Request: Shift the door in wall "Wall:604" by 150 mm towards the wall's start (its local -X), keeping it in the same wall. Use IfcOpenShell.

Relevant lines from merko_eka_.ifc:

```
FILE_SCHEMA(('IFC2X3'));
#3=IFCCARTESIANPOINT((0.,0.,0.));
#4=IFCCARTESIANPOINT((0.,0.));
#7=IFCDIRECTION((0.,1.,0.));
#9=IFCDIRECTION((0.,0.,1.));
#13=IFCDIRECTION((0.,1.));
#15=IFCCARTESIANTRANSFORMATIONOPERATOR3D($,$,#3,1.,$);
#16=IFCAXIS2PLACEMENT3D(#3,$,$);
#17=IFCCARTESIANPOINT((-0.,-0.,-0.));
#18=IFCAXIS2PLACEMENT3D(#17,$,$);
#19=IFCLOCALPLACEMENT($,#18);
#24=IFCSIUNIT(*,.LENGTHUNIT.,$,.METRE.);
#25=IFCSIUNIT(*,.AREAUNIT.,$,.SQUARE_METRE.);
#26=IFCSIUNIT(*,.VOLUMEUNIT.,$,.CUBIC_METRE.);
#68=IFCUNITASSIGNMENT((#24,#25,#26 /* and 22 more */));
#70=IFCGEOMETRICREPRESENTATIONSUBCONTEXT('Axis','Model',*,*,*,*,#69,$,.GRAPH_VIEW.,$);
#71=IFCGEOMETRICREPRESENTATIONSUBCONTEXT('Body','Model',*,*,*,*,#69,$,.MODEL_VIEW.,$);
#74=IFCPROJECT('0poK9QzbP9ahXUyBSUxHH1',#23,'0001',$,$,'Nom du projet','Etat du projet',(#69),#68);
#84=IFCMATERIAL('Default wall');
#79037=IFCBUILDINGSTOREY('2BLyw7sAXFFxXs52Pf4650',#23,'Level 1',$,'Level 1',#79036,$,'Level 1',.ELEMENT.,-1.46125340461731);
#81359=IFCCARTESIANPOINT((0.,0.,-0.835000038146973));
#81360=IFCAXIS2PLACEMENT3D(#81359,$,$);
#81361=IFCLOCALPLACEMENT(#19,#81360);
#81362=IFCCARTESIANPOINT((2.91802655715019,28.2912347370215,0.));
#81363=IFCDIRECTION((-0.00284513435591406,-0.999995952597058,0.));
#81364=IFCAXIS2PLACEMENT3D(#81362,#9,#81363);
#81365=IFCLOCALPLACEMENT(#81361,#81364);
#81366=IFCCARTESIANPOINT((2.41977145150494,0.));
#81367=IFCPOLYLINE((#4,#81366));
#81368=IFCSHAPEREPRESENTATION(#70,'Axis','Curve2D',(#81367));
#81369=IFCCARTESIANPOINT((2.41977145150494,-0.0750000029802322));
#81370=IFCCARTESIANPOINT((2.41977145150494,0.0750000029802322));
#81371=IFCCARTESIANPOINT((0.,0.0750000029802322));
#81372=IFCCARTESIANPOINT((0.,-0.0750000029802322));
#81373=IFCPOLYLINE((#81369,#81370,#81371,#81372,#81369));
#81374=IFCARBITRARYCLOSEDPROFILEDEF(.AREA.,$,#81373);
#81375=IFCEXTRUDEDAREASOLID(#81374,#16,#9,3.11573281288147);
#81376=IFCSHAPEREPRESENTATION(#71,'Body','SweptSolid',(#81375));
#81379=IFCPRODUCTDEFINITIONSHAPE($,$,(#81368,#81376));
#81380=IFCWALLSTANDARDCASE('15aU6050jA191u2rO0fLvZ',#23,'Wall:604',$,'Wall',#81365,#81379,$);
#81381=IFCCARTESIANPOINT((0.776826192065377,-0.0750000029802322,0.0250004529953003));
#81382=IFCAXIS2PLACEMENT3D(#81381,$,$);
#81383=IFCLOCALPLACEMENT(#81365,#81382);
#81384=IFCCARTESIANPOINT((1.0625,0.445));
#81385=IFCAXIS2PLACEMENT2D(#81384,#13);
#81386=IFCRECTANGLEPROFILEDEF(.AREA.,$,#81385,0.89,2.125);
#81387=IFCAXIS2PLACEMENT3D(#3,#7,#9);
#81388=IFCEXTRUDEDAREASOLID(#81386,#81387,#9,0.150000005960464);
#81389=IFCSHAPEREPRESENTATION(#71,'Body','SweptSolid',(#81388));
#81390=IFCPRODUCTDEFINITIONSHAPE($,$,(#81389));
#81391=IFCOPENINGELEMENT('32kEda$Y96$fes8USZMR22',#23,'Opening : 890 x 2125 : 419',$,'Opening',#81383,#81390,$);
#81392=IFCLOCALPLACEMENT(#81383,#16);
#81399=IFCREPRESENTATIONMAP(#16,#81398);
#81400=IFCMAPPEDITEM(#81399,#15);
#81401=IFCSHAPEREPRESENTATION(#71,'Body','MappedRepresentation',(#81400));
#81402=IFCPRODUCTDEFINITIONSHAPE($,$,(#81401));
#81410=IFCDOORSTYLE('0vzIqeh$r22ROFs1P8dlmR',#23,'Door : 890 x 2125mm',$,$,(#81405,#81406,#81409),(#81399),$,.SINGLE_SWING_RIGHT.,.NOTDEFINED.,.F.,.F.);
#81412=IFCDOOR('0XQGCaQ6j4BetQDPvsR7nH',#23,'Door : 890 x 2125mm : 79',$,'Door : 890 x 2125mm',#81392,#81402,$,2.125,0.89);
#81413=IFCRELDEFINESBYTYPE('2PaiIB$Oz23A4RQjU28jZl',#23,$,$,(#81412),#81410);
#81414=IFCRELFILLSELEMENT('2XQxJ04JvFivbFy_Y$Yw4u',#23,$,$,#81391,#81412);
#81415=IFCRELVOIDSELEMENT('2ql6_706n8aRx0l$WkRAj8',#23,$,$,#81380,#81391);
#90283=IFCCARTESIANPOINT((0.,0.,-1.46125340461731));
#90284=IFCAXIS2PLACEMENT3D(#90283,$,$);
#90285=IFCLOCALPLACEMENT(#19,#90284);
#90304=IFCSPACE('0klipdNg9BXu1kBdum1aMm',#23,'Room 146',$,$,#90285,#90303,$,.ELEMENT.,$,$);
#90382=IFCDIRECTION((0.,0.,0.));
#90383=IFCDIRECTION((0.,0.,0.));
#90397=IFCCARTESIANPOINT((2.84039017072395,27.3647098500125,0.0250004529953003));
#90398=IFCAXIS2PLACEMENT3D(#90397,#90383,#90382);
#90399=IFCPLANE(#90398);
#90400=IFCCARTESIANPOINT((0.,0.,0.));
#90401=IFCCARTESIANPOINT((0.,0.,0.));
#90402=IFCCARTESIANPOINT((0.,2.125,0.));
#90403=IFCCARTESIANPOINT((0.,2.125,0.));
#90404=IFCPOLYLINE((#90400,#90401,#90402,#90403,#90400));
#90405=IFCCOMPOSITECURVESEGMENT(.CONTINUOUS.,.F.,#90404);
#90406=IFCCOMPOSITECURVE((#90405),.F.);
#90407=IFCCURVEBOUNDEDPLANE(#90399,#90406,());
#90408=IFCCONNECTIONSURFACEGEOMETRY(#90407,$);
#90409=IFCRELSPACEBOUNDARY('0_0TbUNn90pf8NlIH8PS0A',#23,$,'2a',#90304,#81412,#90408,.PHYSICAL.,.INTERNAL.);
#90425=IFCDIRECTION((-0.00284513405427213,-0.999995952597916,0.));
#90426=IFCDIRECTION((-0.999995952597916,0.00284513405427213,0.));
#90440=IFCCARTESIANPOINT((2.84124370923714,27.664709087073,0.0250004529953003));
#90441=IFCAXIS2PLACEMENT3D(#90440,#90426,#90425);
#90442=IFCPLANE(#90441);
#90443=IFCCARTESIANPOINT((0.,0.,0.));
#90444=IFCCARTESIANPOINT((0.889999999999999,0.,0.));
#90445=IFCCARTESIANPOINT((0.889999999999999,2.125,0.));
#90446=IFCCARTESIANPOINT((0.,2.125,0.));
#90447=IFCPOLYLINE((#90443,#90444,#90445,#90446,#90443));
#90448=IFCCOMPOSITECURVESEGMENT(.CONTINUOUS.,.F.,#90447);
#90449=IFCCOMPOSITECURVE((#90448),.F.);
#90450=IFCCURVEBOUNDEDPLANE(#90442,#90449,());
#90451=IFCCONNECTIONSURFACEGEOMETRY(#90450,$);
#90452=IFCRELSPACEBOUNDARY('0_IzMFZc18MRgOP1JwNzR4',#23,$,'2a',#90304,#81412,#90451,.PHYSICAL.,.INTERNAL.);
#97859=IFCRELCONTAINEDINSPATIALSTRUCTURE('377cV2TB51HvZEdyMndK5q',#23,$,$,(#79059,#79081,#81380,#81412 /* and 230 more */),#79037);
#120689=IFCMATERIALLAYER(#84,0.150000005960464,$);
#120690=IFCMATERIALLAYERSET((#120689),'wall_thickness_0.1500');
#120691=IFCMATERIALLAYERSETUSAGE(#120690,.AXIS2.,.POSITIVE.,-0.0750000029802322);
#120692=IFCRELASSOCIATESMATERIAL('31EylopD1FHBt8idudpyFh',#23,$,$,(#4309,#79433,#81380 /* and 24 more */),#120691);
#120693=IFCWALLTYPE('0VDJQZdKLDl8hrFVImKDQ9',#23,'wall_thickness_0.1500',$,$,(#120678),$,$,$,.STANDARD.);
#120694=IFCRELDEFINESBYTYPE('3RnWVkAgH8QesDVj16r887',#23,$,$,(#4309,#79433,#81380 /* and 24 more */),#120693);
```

```python
import numpy as np
import ifcopenshell
import ifcopenshell.api.geometry
import ifcopenshell.util.placement

model = ifcopenshell.open("merko_eka_.ifc")

door = model.by_guid("0XQGCaQ6j4BetQDPvsR7nH")
opening = door.FillsVoids[0].RelatingOpeningElement
wall = opening.VoidsElements[0].RelatingBuildingElement

wall_matrix = ifcopenshell.util.placement.get_local_placement(wall.ObjectPlacement)
shift = wall_matrix[:3, 0] * -0.15
before = ifcopenshell.util.placement.get_local_placement(door.ObjectPlacement)[:3, 3].copy()

# The door is placed relative to its opening, so it follows when the opening moves.
matrix = ifcopenshell.util.placement.get_local_placement(opening.ObjectPlacement)
matrix[:3, 3] += shift
ifcopenshell.api.geometry.edit_object_placement(
    model, product=opening, matrix=matrix, is_si=False, should_transform_children=True
)

# Space boundary surfaces are stored in each space's coordinates; move them too.
for rel in door.ProvidesBoundaries:
    if not rel.ConnectionGeometry:
        continue
    surface = rel.ConnectionGeometry.SurfaceOnRelatingElement.BasisSurface
    space_matrix = ifcopenshell.util.placement.get_local_placement(rel.RelatingSpace.ObjectPlacement)
    point = np.array(surface.Position.Location.Coordinates) + space_matrix[:3, :3].T @ shift
    surface.Position = model.createIfcAxis2Placement3D(
        model.createIfcCartesianPoint(point.tolist()), surface.Position.Axis, surface.Position.RefDirection
    )

after = ifcopenshell.util.placement.get_local_placement(door.ObjectPlacement)[:3, 3]
print("door moved by", (after - before).round(3) + 0.0)

model.write("merko_eka__edited.ifc")
```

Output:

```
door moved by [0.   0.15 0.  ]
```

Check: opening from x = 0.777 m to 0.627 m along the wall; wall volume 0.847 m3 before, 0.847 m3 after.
